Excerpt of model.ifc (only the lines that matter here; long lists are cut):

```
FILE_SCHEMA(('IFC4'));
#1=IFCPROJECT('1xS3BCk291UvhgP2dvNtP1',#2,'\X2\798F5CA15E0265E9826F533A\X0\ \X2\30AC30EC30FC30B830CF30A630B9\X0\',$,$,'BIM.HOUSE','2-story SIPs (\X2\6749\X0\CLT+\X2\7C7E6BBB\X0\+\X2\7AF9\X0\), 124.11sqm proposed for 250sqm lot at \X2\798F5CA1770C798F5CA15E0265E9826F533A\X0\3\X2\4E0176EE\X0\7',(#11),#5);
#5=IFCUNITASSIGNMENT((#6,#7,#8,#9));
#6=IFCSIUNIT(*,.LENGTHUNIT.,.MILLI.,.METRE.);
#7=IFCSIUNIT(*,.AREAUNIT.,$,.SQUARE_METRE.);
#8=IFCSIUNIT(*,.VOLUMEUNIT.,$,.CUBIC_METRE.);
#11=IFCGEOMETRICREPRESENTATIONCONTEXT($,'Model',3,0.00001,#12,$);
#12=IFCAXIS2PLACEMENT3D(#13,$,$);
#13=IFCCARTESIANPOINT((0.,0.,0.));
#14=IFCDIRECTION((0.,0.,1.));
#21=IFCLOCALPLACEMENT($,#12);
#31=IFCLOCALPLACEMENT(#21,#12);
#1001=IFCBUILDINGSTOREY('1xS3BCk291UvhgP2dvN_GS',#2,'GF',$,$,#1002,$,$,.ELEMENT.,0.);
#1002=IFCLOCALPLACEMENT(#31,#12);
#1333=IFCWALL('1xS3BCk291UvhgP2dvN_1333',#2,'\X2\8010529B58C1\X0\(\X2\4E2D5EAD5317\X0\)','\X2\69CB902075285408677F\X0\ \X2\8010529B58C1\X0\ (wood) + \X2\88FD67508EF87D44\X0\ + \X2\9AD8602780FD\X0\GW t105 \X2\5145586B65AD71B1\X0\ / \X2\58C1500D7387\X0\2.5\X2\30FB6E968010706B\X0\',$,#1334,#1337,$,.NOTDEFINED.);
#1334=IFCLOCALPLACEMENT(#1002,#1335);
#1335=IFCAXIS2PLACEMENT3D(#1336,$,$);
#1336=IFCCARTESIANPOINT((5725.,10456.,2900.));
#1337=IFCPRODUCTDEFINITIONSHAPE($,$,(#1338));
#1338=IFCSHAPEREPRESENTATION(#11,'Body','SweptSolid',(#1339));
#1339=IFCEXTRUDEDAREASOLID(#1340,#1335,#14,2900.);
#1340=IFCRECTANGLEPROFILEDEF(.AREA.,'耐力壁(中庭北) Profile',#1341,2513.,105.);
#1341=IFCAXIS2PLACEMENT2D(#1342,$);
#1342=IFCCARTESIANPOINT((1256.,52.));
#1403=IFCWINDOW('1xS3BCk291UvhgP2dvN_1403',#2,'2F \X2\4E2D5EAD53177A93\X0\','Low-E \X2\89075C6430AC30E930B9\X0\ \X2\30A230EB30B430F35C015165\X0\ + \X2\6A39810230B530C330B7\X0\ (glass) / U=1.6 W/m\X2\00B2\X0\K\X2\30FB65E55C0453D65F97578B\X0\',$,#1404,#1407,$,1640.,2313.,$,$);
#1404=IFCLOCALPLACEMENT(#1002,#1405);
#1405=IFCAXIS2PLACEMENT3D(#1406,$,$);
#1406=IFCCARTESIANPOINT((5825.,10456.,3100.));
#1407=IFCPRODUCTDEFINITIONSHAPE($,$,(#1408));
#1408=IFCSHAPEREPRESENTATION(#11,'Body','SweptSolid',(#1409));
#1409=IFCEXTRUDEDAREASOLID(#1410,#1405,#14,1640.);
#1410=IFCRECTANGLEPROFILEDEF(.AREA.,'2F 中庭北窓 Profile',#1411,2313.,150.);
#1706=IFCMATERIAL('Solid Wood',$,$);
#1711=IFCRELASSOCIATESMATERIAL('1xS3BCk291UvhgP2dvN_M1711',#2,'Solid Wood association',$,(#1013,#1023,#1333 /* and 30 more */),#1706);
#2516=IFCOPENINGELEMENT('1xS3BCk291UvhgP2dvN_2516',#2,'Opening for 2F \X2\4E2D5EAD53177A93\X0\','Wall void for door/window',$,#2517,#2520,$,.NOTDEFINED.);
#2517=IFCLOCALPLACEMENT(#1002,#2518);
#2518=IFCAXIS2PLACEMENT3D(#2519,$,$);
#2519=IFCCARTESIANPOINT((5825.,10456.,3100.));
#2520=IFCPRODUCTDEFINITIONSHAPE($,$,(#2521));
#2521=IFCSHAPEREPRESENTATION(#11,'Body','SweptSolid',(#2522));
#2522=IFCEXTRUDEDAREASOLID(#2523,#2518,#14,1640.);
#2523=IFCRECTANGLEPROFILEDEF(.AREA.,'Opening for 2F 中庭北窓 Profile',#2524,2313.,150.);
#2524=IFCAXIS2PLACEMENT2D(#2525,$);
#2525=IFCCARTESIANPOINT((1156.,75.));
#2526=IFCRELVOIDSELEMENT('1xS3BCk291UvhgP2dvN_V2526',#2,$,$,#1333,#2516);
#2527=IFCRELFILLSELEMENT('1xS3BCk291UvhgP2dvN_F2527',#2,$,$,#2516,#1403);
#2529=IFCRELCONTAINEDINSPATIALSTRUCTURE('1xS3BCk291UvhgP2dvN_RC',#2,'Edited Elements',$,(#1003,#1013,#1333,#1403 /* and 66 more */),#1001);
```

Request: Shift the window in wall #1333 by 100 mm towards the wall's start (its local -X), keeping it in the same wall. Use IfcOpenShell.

```python
import ifcopenshell
import ifcopenshell.api.geometry
import ifcopenshell.util.placement
import ifcopenshell.util.unit

model = ifcopenshell.open("model.ifc")
unit_scale = ifcopenshell.util.unit.calculate_unit_scale(model)

window = model.by_id(1403)
opening = window.FillsVoids[0].RelatingOpeningElement
wall = opening.VoidsElements[0].RelatingBuildingElement

wall_matrix = ifcopenshell.util.placement.get_local_placement(wall.ObjectPlacement)
shift = wall_matrix[:3, 0] * -0.1 / unit_scale
before = ifcopenshell.util.placement.get_local_placement(window.ObjectPlacement)[:3, 3].copy()

# The window is not placed relative to its opening, so move both.
for product in (opening, window):
    matrix = ifcopenshell.util.placement.get_local_placement(product.ObjectPlacement)
    matrix[:3, 3] += shift
    ifcopenshell.api.geometry.edit_object_placement(model, product=product, matrix=matrix, is_si=False)

after = ifcopenshell.util.placement.get_local_placement(window.ObjectPlacement)[:3, 3]
print("window moved by", (after - before).round(3) + 0.0)

model.write("model_edited.ifc")
```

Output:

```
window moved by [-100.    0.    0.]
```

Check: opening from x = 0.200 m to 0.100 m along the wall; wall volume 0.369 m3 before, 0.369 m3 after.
